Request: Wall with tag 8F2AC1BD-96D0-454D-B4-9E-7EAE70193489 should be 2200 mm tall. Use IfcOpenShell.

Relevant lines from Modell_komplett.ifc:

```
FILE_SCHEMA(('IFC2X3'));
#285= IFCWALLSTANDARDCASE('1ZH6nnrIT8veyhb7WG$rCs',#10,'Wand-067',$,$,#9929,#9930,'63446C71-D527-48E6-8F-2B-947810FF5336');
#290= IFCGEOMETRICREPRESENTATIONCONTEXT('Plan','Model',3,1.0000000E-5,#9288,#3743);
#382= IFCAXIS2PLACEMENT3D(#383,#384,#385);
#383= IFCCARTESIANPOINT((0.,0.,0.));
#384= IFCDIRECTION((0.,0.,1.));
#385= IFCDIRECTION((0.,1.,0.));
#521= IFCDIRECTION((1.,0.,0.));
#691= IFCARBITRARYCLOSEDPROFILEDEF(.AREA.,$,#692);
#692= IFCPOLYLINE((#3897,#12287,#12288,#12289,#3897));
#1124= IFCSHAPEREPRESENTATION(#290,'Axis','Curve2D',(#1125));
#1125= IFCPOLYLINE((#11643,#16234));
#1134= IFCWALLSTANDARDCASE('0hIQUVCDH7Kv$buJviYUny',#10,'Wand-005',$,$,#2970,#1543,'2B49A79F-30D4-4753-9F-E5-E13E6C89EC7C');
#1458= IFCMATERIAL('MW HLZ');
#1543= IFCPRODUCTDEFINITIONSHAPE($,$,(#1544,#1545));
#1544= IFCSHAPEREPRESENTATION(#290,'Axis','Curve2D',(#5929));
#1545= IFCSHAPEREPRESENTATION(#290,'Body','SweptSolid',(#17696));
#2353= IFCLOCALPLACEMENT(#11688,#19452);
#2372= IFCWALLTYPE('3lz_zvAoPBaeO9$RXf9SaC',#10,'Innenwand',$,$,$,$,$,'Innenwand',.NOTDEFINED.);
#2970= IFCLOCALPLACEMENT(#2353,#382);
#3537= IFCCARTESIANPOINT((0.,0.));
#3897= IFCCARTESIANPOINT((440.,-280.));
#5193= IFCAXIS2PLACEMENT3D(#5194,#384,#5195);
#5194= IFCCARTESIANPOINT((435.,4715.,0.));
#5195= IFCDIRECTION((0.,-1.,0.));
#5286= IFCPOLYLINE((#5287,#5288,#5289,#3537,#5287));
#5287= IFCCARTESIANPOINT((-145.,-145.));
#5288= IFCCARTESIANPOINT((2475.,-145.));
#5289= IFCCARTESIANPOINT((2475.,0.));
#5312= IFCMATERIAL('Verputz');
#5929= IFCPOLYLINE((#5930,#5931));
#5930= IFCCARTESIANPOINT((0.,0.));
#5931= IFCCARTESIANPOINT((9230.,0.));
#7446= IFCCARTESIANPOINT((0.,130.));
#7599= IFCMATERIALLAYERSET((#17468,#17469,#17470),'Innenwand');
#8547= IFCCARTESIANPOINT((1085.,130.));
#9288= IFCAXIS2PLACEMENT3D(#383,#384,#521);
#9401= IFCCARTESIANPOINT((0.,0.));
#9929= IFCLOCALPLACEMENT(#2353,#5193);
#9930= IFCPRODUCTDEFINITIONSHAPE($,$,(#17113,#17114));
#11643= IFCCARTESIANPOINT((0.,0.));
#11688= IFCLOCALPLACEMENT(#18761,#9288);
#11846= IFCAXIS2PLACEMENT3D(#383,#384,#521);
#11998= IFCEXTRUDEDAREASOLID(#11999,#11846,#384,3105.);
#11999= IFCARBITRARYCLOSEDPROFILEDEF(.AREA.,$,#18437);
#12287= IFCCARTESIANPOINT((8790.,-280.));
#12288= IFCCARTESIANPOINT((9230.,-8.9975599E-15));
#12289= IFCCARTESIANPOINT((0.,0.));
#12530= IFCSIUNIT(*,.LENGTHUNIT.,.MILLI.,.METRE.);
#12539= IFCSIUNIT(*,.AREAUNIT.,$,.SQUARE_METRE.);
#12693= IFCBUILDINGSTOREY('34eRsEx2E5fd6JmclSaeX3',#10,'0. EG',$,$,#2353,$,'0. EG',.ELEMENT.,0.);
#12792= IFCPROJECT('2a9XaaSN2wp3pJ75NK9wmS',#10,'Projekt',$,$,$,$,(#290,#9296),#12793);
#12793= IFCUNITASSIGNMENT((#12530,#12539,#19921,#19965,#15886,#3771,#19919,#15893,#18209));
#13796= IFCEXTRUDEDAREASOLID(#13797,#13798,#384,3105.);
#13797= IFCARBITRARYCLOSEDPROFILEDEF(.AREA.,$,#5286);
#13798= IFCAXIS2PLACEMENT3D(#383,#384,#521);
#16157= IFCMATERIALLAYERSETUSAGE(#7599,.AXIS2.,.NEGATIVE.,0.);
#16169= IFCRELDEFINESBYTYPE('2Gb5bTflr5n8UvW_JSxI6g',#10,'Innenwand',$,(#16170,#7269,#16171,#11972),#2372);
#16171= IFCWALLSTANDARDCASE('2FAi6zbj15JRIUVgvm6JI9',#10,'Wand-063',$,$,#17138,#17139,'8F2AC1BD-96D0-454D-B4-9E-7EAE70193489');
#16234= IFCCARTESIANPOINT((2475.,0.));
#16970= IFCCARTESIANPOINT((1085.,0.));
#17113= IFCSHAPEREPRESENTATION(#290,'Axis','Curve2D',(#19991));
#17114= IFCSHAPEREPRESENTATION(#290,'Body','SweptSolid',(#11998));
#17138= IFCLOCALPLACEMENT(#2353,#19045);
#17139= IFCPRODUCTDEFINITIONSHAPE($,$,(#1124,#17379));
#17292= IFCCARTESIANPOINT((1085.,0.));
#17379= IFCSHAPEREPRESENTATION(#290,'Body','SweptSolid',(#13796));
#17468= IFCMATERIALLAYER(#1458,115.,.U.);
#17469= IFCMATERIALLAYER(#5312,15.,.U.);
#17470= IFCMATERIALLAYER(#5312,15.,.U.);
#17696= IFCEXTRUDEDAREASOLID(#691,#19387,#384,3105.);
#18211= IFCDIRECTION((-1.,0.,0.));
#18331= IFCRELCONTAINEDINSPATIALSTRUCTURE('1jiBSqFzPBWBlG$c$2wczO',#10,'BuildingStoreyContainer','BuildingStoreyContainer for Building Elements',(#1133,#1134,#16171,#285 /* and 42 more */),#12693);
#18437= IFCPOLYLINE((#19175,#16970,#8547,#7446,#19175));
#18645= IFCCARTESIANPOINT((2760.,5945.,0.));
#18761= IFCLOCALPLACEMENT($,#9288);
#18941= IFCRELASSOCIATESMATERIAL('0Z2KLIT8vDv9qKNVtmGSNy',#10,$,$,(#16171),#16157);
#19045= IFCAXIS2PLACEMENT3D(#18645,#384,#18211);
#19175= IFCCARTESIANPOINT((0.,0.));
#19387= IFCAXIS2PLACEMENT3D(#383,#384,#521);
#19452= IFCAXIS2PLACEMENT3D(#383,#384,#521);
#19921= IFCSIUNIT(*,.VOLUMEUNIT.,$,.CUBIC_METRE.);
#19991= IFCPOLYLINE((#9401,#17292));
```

```python
import ifcopenshell
import ifcopenshell.geom
import ifcopenshell.util.shape
import ifcopenshell.util.unit

model = ifcopenshell.open("Modell_komplett.ifc")
unit_scale = ifcopenshell.util.unit.calculate_unit_scale(model)
settings = ifcopenshell.geom.settings()


def volume(element):
    """Net volume in cubic metres, openings subtracted."""
    shape = ifcopenshell.geom.create_shape(settings, element)
    return ifcopenshell.util.shape.get_volume(shape.geometry)


wall = model.by_id(16171)
before = volume(wall)

body = next(r for r in wall.Representation.Representations if r.RepresentationIdentifier == "Body")
solid = body.Items[0]
old_height = solid.Depth
solid.Depth = 2.2 / unit_scale
after = volume(wall)

print(f"height {old_height:g} -> {solid.Depth:g}, volume {before:.3f} -> {after:.3f} m3")

model.write("Modell_komplett_v2.ifc")
```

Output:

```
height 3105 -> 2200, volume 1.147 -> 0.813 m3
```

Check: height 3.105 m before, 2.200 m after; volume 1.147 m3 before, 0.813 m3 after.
